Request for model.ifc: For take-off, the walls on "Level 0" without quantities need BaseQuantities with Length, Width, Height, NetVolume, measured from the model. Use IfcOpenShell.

First a look at what the model holds.

```python
import ifcopenshell
import ifcopenshell.util.element
import ifcopenshell.util.unit

model = ifcopenshell.open("model.ifc")
print(model.schema)
for unit_type in ("LENGTHUNIT", "AREAUNIT", "VOLUMEUNIT"):
    print(unit_type, ifcopenshell.util.unit.calculate_unit_scale(model, unit_type))
storey = next(s for s in model.by_type("IfcBuildingStorey") if s.Name == "Level 0")
walls = [e for e in ifcopenshell.util.element.get_decomposition(storey) if e.is_a("IfcWall")]
for e in sorted(walls, key=lambda e: e.id()):
    print(e.id(), e.is_a(), e.Name, list(ifcopenshell.util.element.get_psets(e, qtos_only=True)), sep=" | ")
```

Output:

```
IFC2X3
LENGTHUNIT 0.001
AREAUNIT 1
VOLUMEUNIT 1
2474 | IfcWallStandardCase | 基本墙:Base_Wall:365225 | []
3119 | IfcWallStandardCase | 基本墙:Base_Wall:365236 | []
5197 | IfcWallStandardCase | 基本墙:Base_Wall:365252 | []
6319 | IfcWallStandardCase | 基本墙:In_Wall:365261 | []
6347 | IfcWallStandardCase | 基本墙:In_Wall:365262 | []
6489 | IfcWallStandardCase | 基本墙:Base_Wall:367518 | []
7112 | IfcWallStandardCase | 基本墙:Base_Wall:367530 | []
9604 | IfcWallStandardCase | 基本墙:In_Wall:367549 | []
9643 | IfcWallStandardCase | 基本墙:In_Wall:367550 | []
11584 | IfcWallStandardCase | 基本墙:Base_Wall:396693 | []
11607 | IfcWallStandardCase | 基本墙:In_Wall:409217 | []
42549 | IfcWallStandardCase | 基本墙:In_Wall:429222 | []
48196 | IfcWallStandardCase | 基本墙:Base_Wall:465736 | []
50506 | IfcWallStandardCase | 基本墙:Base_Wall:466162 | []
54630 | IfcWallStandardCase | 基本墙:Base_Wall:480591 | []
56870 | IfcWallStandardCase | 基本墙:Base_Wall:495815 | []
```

```python
import ifcopenshell
import ifcopenshell.api.pset
import ifcopenshell.geom
import ifcopenshell.util.element
import ifcopenshell.util.shape
import ifcopenshell.util.unit

model = ifcopenshell.open("model.ifc")
unit_scale = ifcopenshell.util.unit.calculate_unit_scale(model)
volume_scale = ifcopenshell.util.unit.calculate_unit_scale(model, "VOLUMEUNIT")
settings = ifcopenshell.geom.settings()

storey = next(s for s in model.by_type("IfcBuildingStorey") if s.Name == "Level 0")
walls = [e for e in ifcopenshell.util.element.get_decomposition(storey) if e.is_a("IfcWall")]

for e in sorted(walls, key=lambda e: e.id()):
    if ifcopenshell.util.element.get_psets(e, qtos_only=True, should_inherit=False):
        continue
    # Geometry comes back in metres, in the element's own axes.
    shape = ifcopenshell.geom.create_shape(settings, e)
    values = {
        "Length": ifcopenshell.util.shape.get_x(shape.geometry) / unit_scale,
        "Width": ifcopenshell.util.shape.get_y(shape.geometry) / unit_scale,
        "Height": ifcopenshell.util.shape.get_z(shape.geometry) / unit_scale,
        "NetVolume": ifcopenshell.util.shape.get_volume(shape.geometry) / volume_scale,
    }
    qto = ifcopenshell.api.pset.add_qto(model, product=e, name="BaseQuantities")
    ifcopenshell.api.pset.edit_qto(model, qto=qto, properties=values)
    print(e.id(), {k: round(v, 3) for k, v in values.items()})

model.write("model_v2.ifc")
```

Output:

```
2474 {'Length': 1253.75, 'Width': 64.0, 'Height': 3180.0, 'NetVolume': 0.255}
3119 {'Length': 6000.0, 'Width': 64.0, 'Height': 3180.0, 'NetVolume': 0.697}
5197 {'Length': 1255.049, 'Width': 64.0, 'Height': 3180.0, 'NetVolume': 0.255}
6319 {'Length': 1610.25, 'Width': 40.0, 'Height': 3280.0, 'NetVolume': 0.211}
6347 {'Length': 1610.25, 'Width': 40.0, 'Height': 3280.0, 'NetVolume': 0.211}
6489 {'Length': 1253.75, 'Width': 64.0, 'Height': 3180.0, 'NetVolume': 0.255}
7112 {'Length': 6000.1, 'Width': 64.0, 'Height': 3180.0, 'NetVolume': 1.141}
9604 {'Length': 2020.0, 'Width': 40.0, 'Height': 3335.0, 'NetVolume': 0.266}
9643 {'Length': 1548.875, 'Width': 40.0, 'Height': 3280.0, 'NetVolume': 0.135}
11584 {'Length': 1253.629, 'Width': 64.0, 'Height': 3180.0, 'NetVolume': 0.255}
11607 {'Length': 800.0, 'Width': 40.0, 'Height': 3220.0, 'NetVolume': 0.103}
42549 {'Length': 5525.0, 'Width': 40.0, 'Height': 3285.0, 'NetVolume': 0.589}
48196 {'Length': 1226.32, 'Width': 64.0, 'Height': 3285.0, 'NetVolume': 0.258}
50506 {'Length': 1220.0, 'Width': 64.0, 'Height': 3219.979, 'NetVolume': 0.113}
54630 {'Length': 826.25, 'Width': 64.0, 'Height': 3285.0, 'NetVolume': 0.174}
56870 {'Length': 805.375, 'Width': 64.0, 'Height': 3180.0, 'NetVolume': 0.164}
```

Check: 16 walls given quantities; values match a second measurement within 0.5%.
